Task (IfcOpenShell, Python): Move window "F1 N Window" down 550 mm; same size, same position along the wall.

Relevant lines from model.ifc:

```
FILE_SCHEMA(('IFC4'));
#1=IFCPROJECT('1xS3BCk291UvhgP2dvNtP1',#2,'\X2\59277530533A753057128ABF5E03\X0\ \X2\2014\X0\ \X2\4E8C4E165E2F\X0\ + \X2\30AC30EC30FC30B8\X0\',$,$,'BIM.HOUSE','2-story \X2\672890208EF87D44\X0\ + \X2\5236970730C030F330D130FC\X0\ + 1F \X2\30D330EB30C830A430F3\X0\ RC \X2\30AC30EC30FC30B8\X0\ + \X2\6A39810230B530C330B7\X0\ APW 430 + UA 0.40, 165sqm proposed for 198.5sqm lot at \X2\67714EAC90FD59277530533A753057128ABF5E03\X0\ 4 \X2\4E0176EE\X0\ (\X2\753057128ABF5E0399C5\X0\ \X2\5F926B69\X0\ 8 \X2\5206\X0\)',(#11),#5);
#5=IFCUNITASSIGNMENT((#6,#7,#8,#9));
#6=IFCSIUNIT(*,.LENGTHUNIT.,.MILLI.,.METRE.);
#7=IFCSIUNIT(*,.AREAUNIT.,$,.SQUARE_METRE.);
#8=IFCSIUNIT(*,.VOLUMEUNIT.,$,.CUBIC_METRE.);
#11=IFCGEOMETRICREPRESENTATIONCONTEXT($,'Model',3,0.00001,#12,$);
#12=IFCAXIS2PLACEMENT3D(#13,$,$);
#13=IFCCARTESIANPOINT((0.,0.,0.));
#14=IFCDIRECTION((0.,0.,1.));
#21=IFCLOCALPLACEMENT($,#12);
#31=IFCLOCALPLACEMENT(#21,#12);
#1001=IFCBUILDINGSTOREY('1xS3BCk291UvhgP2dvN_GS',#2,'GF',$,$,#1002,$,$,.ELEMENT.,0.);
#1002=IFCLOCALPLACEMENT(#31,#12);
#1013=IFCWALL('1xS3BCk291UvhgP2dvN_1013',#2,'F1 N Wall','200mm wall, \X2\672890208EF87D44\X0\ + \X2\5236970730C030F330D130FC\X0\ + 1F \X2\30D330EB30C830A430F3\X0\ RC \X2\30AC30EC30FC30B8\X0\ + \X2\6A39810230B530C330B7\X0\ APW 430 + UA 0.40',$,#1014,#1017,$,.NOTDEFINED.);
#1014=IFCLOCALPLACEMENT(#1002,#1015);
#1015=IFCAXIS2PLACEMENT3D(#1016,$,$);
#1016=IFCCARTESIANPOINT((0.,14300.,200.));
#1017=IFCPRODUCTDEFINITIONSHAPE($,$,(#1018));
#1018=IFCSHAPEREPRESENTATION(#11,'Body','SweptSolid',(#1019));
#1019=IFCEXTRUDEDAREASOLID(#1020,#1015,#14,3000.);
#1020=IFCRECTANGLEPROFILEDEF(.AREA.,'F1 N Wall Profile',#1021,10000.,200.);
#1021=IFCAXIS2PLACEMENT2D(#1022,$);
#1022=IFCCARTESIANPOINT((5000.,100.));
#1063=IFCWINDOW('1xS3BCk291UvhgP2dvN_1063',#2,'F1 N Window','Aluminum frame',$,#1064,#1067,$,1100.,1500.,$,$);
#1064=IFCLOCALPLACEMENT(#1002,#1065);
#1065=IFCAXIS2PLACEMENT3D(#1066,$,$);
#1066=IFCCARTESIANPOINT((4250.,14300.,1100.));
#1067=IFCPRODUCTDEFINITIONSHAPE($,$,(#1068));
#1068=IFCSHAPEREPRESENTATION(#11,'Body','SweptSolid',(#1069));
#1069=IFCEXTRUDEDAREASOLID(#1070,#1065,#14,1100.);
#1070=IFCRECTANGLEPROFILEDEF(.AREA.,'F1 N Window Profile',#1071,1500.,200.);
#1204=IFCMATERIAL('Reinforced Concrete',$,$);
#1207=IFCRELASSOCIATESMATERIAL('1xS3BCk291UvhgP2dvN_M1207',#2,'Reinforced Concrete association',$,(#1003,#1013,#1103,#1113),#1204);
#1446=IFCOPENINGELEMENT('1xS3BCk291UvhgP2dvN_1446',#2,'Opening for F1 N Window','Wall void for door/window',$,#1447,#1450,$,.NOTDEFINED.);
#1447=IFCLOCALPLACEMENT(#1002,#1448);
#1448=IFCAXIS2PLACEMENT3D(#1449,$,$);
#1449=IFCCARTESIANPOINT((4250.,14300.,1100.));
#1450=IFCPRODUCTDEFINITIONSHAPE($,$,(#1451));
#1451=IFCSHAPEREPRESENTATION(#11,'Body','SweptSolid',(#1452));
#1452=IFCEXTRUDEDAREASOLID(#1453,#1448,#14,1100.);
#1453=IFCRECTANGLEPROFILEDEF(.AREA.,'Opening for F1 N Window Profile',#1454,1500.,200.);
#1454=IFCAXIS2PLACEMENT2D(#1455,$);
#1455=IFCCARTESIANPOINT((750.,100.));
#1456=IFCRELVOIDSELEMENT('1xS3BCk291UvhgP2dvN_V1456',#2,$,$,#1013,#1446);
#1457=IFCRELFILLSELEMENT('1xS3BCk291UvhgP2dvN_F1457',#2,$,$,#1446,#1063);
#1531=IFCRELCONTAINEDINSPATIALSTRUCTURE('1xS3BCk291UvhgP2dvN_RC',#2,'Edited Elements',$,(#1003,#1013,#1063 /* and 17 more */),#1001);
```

```python
import numpy as np
import ifcopenshell
import ifcopenshell.api.geometry
import ifcopenshell.util.placement
import ifcopenshell.util.unit

model = ifcopenshell.open("model.ifc")
unit_scale = ifcopenshell.util.unit.calculate_unit_scale(model)

window = model.by_guid("1xS3BCk291UvhgP2dvN_1063")
opening = window.FillsVoids[0].RelatingOpeningElement
dz = -550.0

shift = np.array([0.0, 0.0, dz])
# The window is not placed relative to its opening, so move both.
for product in (opening, window):
    matrix = ifcopenshell.util.placement.get_local_placement(product.ObjectPlacement)
    matrix[:3, 3] += shift
    ifcopenshell.api.geometry.edit_object_placement(model, product=product, matrix=matrix, is_si=False)

print(f"moved by {dz * unit_scale:+.3f} m")

model.write("model-out.ifc")
```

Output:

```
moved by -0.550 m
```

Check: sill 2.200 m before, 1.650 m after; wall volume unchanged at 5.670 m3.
